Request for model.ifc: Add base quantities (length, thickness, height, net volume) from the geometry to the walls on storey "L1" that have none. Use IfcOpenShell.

First a look at what the model holds.

```python
import ifcopenshell
import ifcopenshell.util.element
import ifcopenshell.util.unit

model = ifcopenshell.open("model.ifc")
print(model.schema)
for unit_type in ("LENGTHUNIT", "AREAUNIT", "VOLUMEUNIT"):
    print(unit_type, ifcopenshell.util.unit.calculate_unit_scale(model, unit_type))
storey = next(s for s in model.by_type("IfcBuildingStorey") if s.Name == "L1")
walls = [e for e in ifcopenshell.util.element.get_decomposition(storey) if e.is_a("IfcWall")]
for e in sorted(walls, key=lambda e: e.id()):
    print(e.id(), e.is_a(), e.Name, list(ifcopenshell.util.element.get_psets(e, qtos_only=True)), sep=" | ")
```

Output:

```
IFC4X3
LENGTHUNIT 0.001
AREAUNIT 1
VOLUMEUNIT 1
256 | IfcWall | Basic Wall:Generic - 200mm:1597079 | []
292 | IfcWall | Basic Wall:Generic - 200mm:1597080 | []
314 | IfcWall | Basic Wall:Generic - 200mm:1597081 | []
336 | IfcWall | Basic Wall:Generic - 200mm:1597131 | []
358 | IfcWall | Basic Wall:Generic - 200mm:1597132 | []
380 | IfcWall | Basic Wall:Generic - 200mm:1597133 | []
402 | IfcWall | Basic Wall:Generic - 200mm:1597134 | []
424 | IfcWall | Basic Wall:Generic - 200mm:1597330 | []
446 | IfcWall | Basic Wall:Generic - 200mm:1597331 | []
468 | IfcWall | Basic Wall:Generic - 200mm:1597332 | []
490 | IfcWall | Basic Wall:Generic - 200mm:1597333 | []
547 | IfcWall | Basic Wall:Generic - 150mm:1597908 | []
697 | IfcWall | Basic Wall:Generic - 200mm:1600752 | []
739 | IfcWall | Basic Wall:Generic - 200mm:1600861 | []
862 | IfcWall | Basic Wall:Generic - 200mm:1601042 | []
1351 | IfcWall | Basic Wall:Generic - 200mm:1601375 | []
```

```python
import ifcopenshell
import ifcopenshell.api.pset
import ifcopenshell.geom
import ifcopenshell.util.element
import ifcopenshell.util.shape
import ifcopenshell.util.unit

model = ifcopenshell.open("model.ifc")
unit_scale = ifcopenshell.util.unit.calculate_unit_scale(model)
volume_scale = ifcopenshell.util.unit.calculate_unit_scale(model, "VOLUMEUNIT")
settings = ifcopenshell.geom.settings()

storey = next(s for s in model.by_type("IfcBuildingStorey") if s.Name == "L1")
walls = [e for e in ifcopenshell.util.element.get_decomposition(storey) if e.is_a("IfcWall")]

for e in sorted(walls, key=lambda e: e.id()):
    if ifcopenshell.util.element.get_psets(e, qtos_only=True, should_inherit=False):
        continue
    # Geometry comes back in metres, in the element's own axes.
    shape = ifcopenshell.geom.create_shape(settings, e)
    values = {
        "Length": ifcopenshell.util.shape.get_x(shape.geometry) / unit_scale,
        "Width": ifcopenshell.util.shape.get_y(shape.geometry) / unit_scale,
        "Height": ifcopenshell.util.shape.get_z(shape.geometry) / unit_scale,
        "NetVolume": ifcopenshell.util.shape.get_volume(shape.geometry) / volume_scale,
    }
    qto = ifcopenshell.api.pset.add_qto(model, product=e, name="Qto_WallBaseQuantities")
    ifcopenshell.api.pset.edit_qto(model, qto=qto, properties=values)
    print(e.id(), {k: round(v, 3) for k, v in values.items()})

model.write("model_v2.ifc")
```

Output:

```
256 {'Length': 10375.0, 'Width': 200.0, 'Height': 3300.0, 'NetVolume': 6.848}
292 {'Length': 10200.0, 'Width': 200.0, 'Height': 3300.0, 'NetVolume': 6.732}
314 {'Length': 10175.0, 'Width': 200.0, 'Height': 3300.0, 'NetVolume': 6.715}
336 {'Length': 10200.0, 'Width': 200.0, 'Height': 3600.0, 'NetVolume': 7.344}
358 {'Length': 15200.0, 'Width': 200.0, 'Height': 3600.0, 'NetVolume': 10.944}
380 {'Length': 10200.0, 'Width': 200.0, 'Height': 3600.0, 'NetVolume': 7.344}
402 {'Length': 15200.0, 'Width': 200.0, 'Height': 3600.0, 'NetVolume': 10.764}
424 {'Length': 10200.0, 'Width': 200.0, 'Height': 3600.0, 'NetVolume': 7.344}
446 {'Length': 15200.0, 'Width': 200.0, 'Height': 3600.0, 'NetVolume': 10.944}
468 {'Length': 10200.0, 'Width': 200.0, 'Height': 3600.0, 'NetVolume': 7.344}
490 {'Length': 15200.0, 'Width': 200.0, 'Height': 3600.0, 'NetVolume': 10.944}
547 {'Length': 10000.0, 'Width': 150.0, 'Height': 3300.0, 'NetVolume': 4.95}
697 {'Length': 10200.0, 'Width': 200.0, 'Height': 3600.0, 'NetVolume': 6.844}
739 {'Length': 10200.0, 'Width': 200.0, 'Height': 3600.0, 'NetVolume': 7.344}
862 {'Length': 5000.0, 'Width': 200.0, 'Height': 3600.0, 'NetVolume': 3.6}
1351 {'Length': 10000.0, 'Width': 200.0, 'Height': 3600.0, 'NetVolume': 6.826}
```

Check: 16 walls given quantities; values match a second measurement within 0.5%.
